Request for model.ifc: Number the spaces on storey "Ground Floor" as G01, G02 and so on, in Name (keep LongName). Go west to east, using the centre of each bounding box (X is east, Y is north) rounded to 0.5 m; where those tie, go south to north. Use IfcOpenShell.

First a look at what the model holds.

```python
import ifcopenshell
import ifcopenshell.util.element
import ifcopenshell.util.placement

model = ifcopenshell.open("model.ifc")
print(model.schema)
storey = next(s for s in model.by_type("IfcBuildingStorey") if s.Name == "Ground Floor")
spaces = [e for e in ifcopenshell.util.element.get_decomposition(storey) if e.is_a("IfcSpace")]
for e in sorted(spaces, key=lambda e: e.id()):
    origin = ifcopenshell.util.placement.get_local_placement(e.ObjectPlacement)[:3, 3]
    print(e.id(), e.Name, e.LongName, origin.round(2) + 0.0, sep=" | ")
```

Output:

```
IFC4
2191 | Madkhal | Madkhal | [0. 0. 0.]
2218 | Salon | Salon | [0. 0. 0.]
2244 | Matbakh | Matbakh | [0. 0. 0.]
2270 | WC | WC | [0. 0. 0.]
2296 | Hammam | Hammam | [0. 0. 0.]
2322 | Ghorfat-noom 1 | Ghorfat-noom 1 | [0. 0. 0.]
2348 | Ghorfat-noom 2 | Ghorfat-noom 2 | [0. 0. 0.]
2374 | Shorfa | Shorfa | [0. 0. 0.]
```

```python
import ifcopenshell
import ifcopenshell.geom
import ifcopenshell.util.element
import ifcopenshell.util.shape

model = ifcopenshell.open("model.ifc")
settings = ifcopenshell.geom.settings()
settings.set("use-world-coords", True)


def centre(element):
    shape = ifcopenshell.geom.create_shape(settings, element)
    return ifcopenshell.util.shape.get_bbox_centroid(shape.geometry)


storey = next(s for s in model.by_type("IfcBuildingStorey") if s.Name == "Ground Floor")
spaces = [e for e in ifcopenshell.util.element.get_decomposition(storey) if e.is_a("IfcSpace")]

# Insertion points can sit at a corner or the storey origin, so sort by the geometry (in metres).
centres = {e: centre(e) for e in spaces}
spaces.sort(key=lambda e: (round(centres[e][0] / 0.5), centres[e][1]))

for i, e in enumerate(spaces, start=1):
    number = f"G{i:02d}"
    e.Name = number
    print(e.id(), number)

model.write("model-out.ifc")
```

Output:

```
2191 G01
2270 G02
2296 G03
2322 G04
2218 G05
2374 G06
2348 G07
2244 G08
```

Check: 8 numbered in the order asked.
